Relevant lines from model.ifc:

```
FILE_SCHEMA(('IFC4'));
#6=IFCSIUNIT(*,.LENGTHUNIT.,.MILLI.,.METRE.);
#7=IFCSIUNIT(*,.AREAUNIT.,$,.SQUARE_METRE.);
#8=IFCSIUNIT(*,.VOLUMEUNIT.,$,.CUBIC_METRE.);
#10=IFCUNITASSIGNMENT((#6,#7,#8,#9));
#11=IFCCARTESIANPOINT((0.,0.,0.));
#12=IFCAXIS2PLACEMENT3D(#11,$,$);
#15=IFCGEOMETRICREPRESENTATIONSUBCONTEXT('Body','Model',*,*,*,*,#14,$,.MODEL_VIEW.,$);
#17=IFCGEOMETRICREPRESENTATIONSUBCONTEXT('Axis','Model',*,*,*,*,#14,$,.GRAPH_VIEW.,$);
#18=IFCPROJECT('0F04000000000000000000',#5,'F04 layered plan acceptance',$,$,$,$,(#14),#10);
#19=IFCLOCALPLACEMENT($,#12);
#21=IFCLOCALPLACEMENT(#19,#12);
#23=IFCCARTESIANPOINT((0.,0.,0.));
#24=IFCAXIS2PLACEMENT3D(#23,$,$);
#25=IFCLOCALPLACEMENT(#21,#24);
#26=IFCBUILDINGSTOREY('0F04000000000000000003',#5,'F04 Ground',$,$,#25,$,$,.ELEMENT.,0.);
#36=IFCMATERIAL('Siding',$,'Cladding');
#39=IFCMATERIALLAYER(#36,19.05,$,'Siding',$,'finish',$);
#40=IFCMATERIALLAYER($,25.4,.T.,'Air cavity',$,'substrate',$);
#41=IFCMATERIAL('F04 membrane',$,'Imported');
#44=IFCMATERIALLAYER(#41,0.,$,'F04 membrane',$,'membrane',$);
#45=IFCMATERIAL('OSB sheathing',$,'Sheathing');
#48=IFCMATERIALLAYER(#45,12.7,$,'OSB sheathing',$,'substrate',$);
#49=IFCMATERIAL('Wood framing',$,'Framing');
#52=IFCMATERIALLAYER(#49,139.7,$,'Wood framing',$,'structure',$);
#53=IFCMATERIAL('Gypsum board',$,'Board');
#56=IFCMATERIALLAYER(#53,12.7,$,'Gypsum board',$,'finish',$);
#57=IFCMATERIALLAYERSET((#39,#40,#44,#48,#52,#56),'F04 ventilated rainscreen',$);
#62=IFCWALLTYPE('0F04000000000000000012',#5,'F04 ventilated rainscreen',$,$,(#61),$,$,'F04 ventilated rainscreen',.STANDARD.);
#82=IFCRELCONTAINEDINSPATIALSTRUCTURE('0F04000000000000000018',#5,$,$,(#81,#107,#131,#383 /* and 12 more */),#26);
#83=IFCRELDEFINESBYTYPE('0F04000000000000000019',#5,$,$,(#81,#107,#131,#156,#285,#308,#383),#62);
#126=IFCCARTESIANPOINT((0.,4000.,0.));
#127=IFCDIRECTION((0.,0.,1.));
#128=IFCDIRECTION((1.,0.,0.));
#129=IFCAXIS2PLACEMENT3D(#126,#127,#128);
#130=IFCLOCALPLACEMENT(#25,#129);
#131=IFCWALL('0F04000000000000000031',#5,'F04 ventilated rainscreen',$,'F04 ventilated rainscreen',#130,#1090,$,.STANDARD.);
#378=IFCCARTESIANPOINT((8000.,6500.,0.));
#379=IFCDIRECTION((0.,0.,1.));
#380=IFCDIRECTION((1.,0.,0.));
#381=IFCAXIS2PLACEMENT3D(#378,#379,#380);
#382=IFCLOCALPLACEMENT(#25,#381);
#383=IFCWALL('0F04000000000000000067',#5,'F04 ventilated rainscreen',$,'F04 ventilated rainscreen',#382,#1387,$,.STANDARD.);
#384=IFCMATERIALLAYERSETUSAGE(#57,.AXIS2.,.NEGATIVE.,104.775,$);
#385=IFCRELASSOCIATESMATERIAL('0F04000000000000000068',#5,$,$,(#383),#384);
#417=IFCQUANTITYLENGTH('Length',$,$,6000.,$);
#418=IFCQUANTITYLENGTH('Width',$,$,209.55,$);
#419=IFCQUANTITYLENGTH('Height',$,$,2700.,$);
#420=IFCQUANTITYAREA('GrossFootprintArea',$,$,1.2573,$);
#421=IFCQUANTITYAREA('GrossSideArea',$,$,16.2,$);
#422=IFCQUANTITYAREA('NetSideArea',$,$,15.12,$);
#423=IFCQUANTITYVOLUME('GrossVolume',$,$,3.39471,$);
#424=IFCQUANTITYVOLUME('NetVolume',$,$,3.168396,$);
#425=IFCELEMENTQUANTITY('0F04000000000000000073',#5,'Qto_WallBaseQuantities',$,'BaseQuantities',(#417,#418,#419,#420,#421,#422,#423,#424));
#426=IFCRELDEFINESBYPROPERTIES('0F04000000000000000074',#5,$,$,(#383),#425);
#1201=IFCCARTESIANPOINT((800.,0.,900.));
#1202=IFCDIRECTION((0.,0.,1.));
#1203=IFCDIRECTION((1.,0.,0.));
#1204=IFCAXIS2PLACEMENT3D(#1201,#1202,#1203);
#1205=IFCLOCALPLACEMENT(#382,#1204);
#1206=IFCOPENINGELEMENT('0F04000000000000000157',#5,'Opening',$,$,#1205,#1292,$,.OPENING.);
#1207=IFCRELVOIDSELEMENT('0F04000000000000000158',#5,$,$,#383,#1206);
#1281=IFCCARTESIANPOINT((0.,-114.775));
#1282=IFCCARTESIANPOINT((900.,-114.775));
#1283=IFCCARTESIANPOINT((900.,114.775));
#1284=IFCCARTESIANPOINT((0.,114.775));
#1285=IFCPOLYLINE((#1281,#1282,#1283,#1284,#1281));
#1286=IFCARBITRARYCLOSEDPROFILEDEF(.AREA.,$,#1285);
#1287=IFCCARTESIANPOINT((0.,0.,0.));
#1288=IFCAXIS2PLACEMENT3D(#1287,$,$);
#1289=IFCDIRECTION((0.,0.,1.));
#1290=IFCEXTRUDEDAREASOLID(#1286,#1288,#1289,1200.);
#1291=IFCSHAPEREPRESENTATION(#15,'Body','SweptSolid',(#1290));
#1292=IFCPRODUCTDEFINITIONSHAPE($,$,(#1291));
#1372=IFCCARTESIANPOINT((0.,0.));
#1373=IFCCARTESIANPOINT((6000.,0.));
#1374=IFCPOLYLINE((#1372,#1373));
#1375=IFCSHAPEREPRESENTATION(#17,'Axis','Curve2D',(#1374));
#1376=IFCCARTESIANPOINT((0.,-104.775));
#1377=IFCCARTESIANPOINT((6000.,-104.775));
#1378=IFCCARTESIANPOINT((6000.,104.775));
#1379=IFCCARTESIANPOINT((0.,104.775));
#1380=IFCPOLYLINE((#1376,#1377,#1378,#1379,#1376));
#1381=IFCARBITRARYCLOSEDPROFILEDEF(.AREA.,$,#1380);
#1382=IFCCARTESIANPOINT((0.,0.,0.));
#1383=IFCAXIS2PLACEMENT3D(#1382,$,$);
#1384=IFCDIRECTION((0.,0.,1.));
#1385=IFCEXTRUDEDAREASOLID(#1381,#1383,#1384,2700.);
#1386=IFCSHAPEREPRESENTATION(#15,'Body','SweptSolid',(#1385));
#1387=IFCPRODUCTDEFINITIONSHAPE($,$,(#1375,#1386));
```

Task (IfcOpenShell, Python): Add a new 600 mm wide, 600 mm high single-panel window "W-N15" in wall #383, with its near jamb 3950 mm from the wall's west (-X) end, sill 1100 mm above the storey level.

```python
import numpy as np
import ifcopenshell
import ifcopenshell.api.feature
import ifcopenshell.api.geometry
import ifcopenshell.api.pset
import ifcopenshell.api.root
import ifcopenshell.api.spatial
import ifcopenshell.geom
import ifcopenshell.util.element
import ifcopenshell.util.placement
import ifcopenshell.util.representation
import ifcopenshell.util.shape
import ifcopenshell.util.unit

model = ifcopenshell.open("model.ifc")
unit_scale = ifcopenshell.util.unit.calculate_unit_scale(model)
area_scale = ifcopenshell.util.unit.calculate_unit_scale(model, "AREAUNIT")
volume_scale = ifcopenshell.util.unit.calculate_unit_scale(model, "VOLUMEUNIT")
settings = ifcopenshell.geom.settings()


def volume(element):
    """Net volume in cubic metres, openings subtracted."""
    shape = ifcopenshell.geom.create_shape(settings, element)
    return ifcopenshell.util.shape.get_volume(shape.geometry)


wall = model.by_guid("0F04000000000000000067")
storey = ifcopenshell.util.element.get_container(wall, ifc_class="IfcBuildingStorey")
context = ifcopenshell.util.representation.get_context(model, "Model", "Body", "MODEL_VIEW")
before = volume(wall)

width, height, from_end, sill = 0.6, 0.6, 3.95, 1.1  # metres

# The wall runs along its own X axis, and the end named is its -X end.
wall_shape = ifcopenshell.geom.create_shape(settings, wall)
x, y, z = ifcopenshell.util.shape.get_vertices(wall_shape.geometry).T
start = x.min() + from_end
face, thickness = float(y.min()), float(y.max() - y.min())
wall_matrix = ifcopenshell.util.placement.get_local_placement(wall.ObjectPlacement)
level = ifcopenshell.util.placement.get_local_placement(storey.ObjectPlacement)[2, 3]


def in_wall(x, y):
    """Placement at x, y metres in the wall's axes, at sill height."""
    matrix = wall_matrix.copy()
    matrix[:, 3] = wall_matrix @ np.array([x / unit_scale, y / unit_scale, 0.0, 1.0])
    matrix[2, 3] = level + sill / unit_scale
    return matrix


# Opening: a box that overshoots both wall faces by 50 mm.
opening = ifcopenshell.api.root.create_entity(model, ifc_class="IfcOpeningElement", predefined_type="OPENING")
box = ifcopenshell.api.geometry.add_wall_representation(
    model, context=context, length=width, height=height, thickness=thickness + 0.1
)
ifcopenshell.api.geometry.assign_representation(model, product=opening, representation=box)
ifcopenshell.api.geometry.edit_object_placement(model, product=opening, matrix=in_wall(start, face - 0.05), is_si=False)
ifcopenshell.api.feature.add_feature(model, feature=opening, element=wall)

window = ifcopenshell.api.root.create_entity(model, ifc_class="IfcWindow", name="W-N15", predefined_type="WINDOW")
window.OverallWidth, window.OverallHeight = width / unit_scale, height / unit_scale
window.PartitioningType = "SINGLE_PANEL"
body = ifcopenshell.api.geometry.add_window_representation(
    model,
    context=context,
    overall_width=window.OverallWidth,
    overall_height=window.OverallHeight,
    partition_type="SINGLE_PANEL",
)
ifcopenshell.api.geometry.assign_representation(model, product=window, representation=body)
ifcopenshell.api.spatial.assign_container(model, products=[window], relating_structure=storey)
ifcopenshell.api.feature.add_filling(model, opening=opening, element=window)

# Centre the window in the wall's thickness.
ifcopenshell.api.geometry.edit_object_placement(model, product=window, matrix=in_wall(start, face), is_si=False)
window_shape = ifcopenshell.geom.create_shape(settings, window)
depth = ifcopenshell.util.shape.get_vertices(window_shape.geometry)[:, 1]
offset = face + thickness / 2 - (depth.min() + depth.max()) / 2
ifcopenshell.api.geometry.edit_object_placement(model, product=window, matrix=in_wall(start, offset), is_si=False)

after = volume(wall)

# Update the wall's stored quantities.
qto = model.by_id(ifcopenshell.util.element.get_pset(wall, "Qto_WallBaseQuantities", should_inherit=False)["id"])
ifcopenshell.api.pset.edit_qto(model, qto=qto, properties={
    "NetSideArea": after / thickness / area_scale,
    "NetVolume": after / volume_scale,
})

print(f"wall volume {before:.3f} -> {after:.3f} m3")

model.write("model_updated.ifc")
```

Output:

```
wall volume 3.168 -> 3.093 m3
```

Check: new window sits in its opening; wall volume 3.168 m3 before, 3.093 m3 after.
